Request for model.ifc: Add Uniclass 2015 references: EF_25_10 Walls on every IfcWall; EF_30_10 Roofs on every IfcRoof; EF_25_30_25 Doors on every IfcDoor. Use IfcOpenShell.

First a look at what the model holds.

```python
import ifcopenshell

model = ifcopenshell.open("model.ifc")
print(model.schema)
print("classifications:", [c.Name for c in model.by_type("IfcClassification")])
for ifc_class in ("IfcDoor", "IfcRoof", "IfcStair", "IfcWall", "IfcWindow"):
    print(ifc_class, len(model.by_type(ifc_class)))
```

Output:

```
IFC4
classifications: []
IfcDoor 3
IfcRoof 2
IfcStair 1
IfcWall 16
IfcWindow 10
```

```python
import ifcopenshell
import ifcopenshell.api.classification

model = ifcopenshell.open("model.ifc")

system = ifcopenshell.api.classification.add_classification(model, classification="Uniclass 2015")

codes = {
    "IfcWall": ("EF_25_10", "Walls"),
    "IfcRoof": ("EF_30_10", "Roofs"),
    "IfcDoor": ("EF_25_30_25", "Doors"),
}
for ifc_class, (code, name) in codes.items():
    products = model.by_type(ifc_class)
    ifcopenshell.api.classification.add_reference(
        model, products=products, classification=system, identification=code, name=name
    )
    print(code, len(products))

model.write("model_rev.ifc")
```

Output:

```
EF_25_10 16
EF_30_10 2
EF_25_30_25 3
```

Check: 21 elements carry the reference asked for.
